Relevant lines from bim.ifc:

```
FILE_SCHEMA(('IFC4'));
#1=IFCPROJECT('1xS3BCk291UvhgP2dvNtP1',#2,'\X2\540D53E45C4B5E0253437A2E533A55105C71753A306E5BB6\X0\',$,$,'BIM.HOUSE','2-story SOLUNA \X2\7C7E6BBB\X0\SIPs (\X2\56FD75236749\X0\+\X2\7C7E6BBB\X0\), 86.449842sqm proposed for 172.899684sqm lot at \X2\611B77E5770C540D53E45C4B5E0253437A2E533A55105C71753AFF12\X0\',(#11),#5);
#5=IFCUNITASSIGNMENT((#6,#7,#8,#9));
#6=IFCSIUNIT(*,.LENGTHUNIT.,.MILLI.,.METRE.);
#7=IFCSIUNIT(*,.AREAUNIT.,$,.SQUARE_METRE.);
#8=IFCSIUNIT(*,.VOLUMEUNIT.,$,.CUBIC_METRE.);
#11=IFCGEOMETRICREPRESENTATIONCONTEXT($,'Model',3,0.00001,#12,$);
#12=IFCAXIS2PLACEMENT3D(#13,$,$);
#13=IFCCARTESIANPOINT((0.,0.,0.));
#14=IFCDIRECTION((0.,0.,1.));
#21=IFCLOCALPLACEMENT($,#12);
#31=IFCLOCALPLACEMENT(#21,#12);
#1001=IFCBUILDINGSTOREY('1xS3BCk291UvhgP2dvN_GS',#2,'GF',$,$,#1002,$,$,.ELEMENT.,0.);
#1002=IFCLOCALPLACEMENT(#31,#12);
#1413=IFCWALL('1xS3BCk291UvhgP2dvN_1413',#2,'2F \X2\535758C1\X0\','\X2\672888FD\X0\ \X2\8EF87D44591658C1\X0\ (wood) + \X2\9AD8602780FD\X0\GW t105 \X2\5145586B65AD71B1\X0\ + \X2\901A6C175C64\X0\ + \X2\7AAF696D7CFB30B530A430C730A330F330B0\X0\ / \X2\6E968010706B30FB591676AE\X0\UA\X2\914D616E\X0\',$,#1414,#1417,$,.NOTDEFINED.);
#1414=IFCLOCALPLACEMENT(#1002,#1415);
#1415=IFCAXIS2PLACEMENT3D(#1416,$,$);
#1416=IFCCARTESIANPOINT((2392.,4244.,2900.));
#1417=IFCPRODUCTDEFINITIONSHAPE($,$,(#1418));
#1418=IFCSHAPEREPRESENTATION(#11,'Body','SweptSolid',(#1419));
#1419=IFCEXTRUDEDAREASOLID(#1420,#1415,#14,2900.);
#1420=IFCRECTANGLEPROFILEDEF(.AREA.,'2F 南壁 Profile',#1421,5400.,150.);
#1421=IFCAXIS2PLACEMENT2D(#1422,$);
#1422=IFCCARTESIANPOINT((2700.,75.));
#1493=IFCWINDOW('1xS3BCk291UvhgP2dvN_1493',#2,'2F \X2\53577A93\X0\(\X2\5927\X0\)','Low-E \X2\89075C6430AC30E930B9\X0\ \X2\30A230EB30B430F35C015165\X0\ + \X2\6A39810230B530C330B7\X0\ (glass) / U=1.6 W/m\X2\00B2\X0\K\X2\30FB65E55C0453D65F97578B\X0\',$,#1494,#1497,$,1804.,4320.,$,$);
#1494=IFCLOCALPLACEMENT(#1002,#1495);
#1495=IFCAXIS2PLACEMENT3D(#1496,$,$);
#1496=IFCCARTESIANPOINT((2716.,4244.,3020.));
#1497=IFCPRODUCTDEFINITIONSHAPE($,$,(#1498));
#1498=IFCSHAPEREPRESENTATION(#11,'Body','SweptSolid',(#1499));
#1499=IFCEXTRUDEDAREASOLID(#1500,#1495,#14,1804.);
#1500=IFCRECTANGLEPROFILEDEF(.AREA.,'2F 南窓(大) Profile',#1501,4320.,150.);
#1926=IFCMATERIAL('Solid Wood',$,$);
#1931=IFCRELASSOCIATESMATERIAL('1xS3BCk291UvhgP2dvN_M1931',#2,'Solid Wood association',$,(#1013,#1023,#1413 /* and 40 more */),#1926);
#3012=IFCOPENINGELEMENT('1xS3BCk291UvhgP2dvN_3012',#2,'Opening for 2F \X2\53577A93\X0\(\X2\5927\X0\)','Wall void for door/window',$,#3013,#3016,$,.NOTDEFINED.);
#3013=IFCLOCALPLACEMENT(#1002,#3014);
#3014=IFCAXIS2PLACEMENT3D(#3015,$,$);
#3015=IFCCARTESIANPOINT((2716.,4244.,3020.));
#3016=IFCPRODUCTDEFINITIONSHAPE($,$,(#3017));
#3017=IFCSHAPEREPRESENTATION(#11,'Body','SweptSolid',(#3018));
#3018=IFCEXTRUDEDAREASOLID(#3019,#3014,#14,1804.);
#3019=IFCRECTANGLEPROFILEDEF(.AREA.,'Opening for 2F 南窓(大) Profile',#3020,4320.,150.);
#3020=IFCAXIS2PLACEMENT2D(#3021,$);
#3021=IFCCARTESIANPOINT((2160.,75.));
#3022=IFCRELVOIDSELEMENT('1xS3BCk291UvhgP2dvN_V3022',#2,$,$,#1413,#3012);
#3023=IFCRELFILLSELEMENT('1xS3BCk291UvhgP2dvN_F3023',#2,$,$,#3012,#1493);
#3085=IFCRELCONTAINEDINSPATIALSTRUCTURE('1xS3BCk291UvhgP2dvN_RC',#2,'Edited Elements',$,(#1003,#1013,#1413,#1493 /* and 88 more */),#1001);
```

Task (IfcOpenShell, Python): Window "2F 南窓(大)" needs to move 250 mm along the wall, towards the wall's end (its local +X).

```python
import ifcopenshell
import ifcopenshell.api.geometry
import ifcopenshell.util.placement
import ifcopenshell.util.unit

model = ifcopenshell.open("bim.ifc")
unit_scale = ifcopenshell.util.unit.calculate_unit_scale(model)

window = model.by_guid("1xS3BCk291UvhgP2dvN_1493")
opening = window.FillsVoids[0].RelatingOpeningElement
wall = opening.VoidsElements[0].RelatingBuildingElement

wall_matrix = ifcopenshell.util.placement.get_local_placement(wall.ObjectPlacement)
shift = wall_matrix[:3, 0] * 0.25 / unit_scale
before = ifcopenshell.util.placement.get_local_placement(window.ObjectPlacement)[:3, 3].copy()

# The window is not placed relative to its opening, so move both.
for product in (opening, window):
    matrix = ifcopenshell.util.placement.get_local_placement(product.ObjectPlacement)
    matrix[:3, 3] += shift
    ifcopenshell.api.geometry.edit_object_placement(model, product=product, matrix=matrix, is_si=False)

after = ifcopenshell.util.placement.get_local_placement(window.ObjectPlacement)[:3, 3]
print("window moved by", (after - before).round(3) + 0.0)

model.write("bim_v2.ifc")
```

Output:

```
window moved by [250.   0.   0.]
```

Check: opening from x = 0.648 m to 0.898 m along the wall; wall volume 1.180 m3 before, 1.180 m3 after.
